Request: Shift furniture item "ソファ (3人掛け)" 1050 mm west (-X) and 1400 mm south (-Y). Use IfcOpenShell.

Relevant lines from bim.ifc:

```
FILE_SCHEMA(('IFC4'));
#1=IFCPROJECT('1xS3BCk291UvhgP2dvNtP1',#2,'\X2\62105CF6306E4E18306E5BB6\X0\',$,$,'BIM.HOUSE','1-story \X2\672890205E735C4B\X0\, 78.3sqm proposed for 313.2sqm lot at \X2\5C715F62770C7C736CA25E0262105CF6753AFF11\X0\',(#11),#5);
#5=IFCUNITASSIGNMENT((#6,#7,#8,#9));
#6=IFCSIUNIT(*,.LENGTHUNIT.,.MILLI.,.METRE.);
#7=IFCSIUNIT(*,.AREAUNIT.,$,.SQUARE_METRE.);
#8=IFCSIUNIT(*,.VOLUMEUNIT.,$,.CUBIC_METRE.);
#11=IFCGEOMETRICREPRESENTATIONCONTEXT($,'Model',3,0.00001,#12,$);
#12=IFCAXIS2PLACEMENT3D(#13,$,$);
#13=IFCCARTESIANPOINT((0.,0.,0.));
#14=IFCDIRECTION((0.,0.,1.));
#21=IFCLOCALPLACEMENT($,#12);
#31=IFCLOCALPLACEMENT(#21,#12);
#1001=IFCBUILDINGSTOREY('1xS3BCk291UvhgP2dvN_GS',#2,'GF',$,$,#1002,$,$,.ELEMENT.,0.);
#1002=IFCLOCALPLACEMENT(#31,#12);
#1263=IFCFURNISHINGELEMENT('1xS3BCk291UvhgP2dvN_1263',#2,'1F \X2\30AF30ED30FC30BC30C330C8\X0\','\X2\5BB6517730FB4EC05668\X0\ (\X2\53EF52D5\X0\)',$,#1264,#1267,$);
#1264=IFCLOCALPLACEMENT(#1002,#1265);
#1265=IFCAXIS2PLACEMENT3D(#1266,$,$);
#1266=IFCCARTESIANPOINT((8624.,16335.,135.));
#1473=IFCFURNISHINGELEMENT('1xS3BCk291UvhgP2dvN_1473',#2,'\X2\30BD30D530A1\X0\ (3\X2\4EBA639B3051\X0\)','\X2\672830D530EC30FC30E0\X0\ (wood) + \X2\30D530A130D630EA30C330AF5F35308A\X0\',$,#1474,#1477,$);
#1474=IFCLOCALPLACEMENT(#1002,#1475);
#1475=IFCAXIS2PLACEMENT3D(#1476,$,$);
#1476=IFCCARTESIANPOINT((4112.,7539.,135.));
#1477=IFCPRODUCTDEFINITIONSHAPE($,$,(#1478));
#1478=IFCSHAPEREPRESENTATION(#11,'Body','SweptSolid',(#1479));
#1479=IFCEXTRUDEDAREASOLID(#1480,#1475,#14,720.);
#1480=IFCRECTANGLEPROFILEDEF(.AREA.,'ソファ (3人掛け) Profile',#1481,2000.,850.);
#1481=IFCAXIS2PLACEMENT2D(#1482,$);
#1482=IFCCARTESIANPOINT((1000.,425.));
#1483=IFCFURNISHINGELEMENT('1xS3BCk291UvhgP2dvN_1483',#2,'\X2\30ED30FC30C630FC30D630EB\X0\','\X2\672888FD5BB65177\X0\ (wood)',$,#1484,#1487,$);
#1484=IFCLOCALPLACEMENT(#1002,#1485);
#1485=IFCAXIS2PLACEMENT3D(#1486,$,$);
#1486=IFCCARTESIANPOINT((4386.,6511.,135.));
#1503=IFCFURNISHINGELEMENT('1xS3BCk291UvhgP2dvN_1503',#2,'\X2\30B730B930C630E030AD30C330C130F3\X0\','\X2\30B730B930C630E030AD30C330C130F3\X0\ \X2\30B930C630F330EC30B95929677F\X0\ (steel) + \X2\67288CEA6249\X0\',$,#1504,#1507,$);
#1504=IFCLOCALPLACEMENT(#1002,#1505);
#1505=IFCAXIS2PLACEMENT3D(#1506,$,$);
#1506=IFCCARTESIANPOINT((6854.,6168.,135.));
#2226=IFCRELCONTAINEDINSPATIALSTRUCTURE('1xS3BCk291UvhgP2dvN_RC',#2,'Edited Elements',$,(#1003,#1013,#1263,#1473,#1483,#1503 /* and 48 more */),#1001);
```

```python
import ifcopenshell
import ifcopenshell.api.geometry
import ifcopenshell.util.placement
import ifcopenshell.util.unit

model = ifcopenshell.open("bim.ifc")
unit_scale = ifcopenshell.util.unit.calculate_unit_scale(model)

item = model.by_id(1473)
matrix = ifcopenshell.util.placement.get_local_placement(item.ObjectPlacement)
matrix[0, 3] -= 1.05 / unit_scale
matrix[1, 3] -= 1.4 / unit_scale
ifcopenshell.api.geometry.edit_object_placement(model, product=item, matrix=matrix, is_si=False)

print(ifcopenshell.util.placement.get_local_placement(item.ObjectPlacement).round(3) + 0.0)

model.write("bim-out.ifc")
```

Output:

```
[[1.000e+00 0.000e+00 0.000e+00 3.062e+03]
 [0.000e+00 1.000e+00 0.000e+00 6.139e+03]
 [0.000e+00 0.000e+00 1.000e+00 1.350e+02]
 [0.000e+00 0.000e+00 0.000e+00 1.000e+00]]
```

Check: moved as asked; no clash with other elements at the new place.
